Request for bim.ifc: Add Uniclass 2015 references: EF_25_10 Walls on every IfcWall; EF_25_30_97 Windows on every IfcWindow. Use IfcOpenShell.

First a look at what the model holds.

```python
import ifcopenshell

model = ifcopenshell.open("bim.ifc")
print(model.schema)
print("classifications:", [c.Name for c in model.by_type("IfcClassification")])
for ifc_class in ("IfcDoor", "IfcRoof", "IfcStair", "IfcWall", "IfcWindow"):
    print(ifc_class, len(model.by_type(ifc_class)))
```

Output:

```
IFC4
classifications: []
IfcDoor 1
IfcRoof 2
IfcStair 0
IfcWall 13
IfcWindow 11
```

```python
import ifcopenshell
import ifcopenshell.api.classification

model = ifcopenshell.open("bim.ifc")

system = ifcopenshell.api.classification.add_classification(model, classification="Uniclass 2015")

codes = {
    "IfcWall": ("EF_25_10", "Walls"),
    "IfcWindow": ("EF_25_30_97", "Windows"),
}
for ifc_class, (code, name) in codes.items():
    products = model.by_type(ifc_class)
    ifcopenshell.api.classification.add_reference(
        model, products=products, classification=system, identification=code, name=name
    )
    print(code, len(products))

model.write("bim_rev.ifc")
```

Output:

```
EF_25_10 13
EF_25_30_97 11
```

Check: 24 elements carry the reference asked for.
